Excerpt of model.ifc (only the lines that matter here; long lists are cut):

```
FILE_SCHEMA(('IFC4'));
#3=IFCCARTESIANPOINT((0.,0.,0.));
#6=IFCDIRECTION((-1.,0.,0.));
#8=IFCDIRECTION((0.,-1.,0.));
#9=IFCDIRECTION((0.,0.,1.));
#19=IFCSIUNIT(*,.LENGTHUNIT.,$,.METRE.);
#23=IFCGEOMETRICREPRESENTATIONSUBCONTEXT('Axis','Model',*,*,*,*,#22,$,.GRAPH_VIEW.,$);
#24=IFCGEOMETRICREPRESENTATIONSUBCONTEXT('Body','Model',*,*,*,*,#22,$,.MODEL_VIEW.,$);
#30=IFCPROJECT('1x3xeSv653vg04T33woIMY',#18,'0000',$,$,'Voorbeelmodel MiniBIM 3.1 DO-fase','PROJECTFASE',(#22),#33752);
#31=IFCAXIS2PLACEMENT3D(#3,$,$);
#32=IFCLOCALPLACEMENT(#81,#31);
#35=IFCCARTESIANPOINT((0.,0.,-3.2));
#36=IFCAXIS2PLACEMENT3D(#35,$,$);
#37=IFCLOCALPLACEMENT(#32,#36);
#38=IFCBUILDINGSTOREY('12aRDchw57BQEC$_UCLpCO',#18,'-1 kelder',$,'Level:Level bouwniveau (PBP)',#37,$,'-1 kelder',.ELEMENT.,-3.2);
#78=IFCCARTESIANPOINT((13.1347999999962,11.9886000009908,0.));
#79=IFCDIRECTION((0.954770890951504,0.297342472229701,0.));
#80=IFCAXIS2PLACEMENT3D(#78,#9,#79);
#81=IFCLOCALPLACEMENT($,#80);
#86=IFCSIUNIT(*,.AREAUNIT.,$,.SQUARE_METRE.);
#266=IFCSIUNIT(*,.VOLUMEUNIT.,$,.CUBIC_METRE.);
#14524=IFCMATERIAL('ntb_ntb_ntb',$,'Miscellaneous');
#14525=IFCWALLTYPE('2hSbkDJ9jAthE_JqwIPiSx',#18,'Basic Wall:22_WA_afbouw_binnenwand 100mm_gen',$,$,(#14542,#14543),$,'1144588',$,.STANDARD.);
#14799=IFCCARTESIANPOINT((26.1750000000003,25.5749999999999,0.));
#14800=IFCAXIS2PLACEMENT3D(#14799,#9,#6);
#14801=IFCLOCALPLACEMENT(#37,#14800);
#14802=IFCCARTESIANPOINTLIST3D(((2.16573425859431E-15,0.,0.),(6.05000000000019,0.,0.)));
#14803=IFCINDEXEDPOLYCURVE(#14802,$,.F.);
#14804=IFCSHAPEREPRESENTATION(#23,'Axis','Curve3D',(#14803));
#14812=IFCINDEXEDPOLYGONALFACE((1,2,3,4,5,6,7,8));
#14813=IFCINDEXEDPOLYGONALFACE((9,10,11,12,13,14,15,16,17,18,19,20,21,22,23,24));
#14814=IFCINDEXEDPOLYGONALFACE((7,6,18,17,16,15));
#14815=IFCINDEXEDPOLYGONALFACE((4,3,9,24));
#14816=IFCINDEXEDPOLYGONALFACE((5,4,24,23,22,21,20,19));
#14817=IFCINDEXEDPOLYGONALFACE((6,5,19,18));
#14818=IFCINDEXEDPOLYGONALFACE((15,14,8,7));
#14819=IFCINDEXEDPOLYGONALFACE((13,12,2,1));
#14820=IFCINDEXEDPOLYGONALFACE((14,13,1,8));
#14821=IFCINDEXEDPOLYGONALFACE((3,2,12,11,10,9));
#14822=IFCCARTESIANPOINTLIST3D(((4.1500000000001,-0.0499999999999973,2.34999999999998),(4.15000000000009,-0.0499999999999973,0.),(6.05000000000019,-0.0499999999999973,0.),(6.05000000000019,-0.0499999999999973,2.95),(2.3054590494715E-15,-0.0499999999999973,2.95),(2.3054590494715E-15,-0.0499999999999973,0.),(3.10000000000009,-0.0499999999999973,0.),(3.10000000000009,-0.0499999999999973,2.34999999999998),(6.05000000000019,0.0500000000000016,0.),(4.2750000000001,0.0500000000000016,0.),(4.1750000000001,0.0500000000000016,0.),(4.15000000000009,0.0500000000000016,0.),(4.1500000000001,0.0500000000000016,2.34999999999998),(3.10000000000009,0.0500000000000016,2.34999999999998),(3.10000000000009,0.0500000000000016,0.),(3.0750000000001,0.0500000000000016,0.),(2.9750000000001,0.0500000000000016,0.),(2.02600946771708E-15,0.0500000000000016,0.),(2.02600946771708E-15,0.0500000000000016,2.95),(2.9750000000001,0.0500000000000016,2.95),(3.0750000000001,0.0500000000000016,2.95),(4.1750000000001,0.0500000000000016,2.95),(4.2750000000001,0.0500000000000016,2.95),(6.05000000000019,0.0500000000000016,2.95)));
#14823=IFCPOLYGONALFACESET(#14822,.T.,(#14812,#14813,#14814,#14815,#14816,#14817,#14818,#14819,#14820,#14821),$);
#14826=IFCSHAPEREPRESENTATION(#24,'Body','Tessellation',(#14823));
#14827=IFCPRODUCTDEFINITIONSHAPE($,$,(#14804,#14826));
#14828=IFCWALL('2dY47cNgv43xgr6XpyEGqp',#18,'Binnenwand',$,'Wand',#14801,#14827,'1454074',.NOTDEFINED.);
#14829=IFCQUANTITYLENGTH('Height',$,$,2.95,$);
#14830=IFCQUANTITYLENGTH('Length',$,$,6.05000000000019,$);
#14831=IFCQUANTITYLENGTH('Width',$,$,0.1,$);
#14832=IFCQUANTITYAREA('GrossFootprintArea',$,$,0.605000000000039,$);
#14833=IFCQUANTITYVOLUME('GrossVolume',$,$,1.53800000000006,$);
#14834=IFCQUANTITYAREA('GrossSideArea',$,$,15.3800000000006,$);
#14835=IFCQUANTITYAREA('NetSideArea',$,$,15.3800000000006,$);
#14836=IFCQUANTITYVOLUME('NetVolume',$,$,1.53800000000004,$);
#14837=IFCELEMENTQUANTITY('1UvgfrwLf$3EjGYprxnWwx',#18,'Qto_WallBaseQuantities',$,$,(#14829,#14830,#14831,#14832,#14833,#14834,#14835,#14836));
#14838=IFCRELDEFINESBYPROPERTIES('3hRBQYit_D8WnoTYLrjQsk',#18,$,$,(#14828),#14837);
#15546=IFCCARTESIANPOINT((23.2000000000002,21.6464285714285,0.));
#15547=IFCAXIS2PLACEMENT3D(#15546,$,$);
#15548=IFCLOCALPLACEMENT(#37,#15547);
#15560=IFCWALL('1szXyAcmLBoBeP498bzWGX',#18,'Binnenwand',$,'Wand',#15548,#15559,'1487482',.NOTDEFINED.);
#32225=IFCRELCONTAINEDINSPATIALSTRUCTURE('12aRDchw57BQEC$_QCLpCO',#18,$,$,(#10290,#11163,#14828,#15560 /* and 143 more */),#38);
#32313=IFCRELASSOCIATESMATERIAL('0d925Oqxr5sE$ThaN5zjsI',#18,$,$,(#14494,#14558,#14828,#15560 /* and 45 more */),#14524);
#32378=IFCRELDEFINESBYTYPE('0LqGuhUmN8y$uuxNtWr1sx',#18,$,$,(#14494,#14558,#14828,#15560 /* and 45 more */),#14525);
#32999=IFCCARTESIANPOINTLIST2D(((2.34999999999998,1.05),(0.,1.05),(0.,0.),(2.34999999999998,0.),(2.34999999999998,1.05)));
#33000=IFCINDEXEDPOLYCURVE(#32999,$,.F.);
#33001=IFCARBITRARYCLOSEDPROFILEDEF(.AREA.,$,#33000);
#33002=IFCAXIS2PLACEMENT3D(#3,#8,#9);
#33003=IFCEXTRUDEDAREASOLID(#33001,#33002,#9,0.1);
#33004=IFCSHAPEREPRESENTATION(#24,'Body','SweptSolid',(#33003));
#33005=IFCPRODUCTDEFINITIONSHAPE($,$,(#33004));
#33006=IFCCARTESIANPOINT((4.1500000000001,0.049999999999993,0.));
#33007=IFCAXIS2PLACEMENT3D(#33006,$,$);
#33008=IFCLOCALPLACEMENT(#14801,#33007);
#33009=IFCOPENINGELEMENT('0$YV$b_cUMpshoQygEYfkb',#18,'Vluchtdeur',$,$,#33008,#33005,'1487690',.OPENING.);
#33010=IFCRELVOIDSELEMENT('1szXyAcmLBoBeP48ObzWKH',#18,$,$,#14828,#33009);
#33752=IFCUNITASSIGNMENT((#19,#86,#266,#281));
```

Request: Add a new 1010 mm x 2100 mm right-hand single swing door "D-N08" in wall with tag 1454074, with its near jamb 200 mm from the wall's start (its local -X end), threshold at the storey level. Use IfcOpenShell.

```python
import numpy as np
import ifcopenshell
import ifcopenshell.api.feature
import ifcopenshell.api.geometry
import ifcopenshell.api.pset
import ifcopenshell.api.root
import ifcopenshell.api.spatial
import ifcopenshell.geom
import ifcopenshell.util.element
import ifcopenshell.util.placement
import ifcopenshell.util.representation
import ifcopenshell.util.shape
import ifcopenshell.util.unit

model = ifcopenshell.open("model.ifc")
unit_scale = ifcopenshell.util.unit.calculate_unit_scale(model)
area_scale = ifcopenshell.util.unit.calculate_unit_scale(model, "AREAUNIT")
volume_scale = ifcopenshell.util.unit.calculate_unit_scale(model, "VOLUMEUNIT")
settings = ifcopenshell.geom.settings()


def volume(element):
    """Net volume in cubic metres, openings subtracted."""
    shape = ifcopenshell.geom.create_shape(settings, element)
    return ifcopenshell.util.shape.get_volume(shape.geometry)


wall = model.by_guid("2dY47cNgv43xgr6XpyEGqp")
storey = ifcopenshell.util.element.get_container(wall, ifc_class="IfcBuildingStorey")
context = ifcopenshell.util.representation.get_context(model, "Model", "Body", "MODEL_VIEW")
before = volume(wall)

width, height, from_end, sill = 1.01, 2.1, 0.2, 0.0  # metres

# The wall runs along its own X axis, and the end named is its -X end.
wall_shape = ifcopenshell.geom.create_shape(settings, wall)
x, y, z = ifcopenshell.util.shape.get_vertices(wall_shape.geometry).T
start = x.min() + from_end
face, thickness = float(y.min()), float(y.max() - y.min())
wall_matrix = ifcopenshell.util.placement.get_local_placement(wall.ObjectPlacement)
level = ifcopenshell.util.placement.get_local_placement(storey.ObjectPlacement)[2, 3]


def in_wall(x, y):
    """Placement at x, y metres in the wall's axes, at sill height."""
    matrix = wall_matrix.copy()
    matrix[:, 3] = wall_matrix @ np.array([x / unit_scale, y / unit_scale, 0.0, 1.0])
    matrix[2, 3] = level + sill / unit_scale
    return matrix


# Opening: a box that overshoots both wall faces by 50 mm.
opening = ifcopenshell.api.root.create_entity(model, ifc_class="IfcOpeningElement", predefined_type="OPENING")
box = ifcopenshell.api.geometry.add_wall_representation(
    model, context=context, length=width, height=height, thickness=thickness + 0.1
)
ifcopenshell.api.geometry.assign_representation(model, product=opening, representation=box)
ifcopenshell.api.geometry.edit_object_placement(model, product=opening, matrix=in_wall(start, face - 0.05), is_si=False)
ifcopenshell.api.feature.add_feature(model, feature=opening, element=wall)

door = ifcopenshell.api.root.create_entity(model, ifc_class="IfcDoor", name="D-N08", predefined_type="DOOR")
door.OverallWidth, door.OverallHeight = width / unit_scale, height / unit_scale
door.OperationType = "SINGLE_SWING_RIGHT"
body = ifcopenshell.api.geometry.add_door_representation(
    model,
    context=context,
    overall_width=door.OverallWidth,
    overall_height=door.OverallHeight,
    operation_type="SINGLE_SWING_RIGHT",
    lining_properties={"LiningDepth": thickness / unit_scale, "ThresholdDepth": thickness / unit_scale},
)
ifcopenshell.api.geometry.assign_representation(model, product=door, representation=body)
ifcopenshell.api.spatial.assign_container(model, products=[door], relating_structure=storey)
ifcopenshell.api.feature.add_filling(model, opening=opening, element=door)

# The lining spans the wall, so the door starts at the wall face.
ifcopenshell.api.geometry.edit_object_placement(model, product=door, matrix=in_wall(start, face), is_si=False)

after = volume(wall)

# Update the wall's stored quantities.
qto = model.by_id(ifcopenshell.util.element.get_pset(wall, "Qto_WallBaseQuantities", should_inherit=False)["id"])
ifcopenshell.api.pset.edit_qto(model, qto=qto, properties={
    "NetSideArea": after / thickness / area_scale,
    "NetVolume": after / volume_scale,
})

print(f"wall volume {before:.3f} -> {after:.3f} m3")

model.write("model-out.ifc")
```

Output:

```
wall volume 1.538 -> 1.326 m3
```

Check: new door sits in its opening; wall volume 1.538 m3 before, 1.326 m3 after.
